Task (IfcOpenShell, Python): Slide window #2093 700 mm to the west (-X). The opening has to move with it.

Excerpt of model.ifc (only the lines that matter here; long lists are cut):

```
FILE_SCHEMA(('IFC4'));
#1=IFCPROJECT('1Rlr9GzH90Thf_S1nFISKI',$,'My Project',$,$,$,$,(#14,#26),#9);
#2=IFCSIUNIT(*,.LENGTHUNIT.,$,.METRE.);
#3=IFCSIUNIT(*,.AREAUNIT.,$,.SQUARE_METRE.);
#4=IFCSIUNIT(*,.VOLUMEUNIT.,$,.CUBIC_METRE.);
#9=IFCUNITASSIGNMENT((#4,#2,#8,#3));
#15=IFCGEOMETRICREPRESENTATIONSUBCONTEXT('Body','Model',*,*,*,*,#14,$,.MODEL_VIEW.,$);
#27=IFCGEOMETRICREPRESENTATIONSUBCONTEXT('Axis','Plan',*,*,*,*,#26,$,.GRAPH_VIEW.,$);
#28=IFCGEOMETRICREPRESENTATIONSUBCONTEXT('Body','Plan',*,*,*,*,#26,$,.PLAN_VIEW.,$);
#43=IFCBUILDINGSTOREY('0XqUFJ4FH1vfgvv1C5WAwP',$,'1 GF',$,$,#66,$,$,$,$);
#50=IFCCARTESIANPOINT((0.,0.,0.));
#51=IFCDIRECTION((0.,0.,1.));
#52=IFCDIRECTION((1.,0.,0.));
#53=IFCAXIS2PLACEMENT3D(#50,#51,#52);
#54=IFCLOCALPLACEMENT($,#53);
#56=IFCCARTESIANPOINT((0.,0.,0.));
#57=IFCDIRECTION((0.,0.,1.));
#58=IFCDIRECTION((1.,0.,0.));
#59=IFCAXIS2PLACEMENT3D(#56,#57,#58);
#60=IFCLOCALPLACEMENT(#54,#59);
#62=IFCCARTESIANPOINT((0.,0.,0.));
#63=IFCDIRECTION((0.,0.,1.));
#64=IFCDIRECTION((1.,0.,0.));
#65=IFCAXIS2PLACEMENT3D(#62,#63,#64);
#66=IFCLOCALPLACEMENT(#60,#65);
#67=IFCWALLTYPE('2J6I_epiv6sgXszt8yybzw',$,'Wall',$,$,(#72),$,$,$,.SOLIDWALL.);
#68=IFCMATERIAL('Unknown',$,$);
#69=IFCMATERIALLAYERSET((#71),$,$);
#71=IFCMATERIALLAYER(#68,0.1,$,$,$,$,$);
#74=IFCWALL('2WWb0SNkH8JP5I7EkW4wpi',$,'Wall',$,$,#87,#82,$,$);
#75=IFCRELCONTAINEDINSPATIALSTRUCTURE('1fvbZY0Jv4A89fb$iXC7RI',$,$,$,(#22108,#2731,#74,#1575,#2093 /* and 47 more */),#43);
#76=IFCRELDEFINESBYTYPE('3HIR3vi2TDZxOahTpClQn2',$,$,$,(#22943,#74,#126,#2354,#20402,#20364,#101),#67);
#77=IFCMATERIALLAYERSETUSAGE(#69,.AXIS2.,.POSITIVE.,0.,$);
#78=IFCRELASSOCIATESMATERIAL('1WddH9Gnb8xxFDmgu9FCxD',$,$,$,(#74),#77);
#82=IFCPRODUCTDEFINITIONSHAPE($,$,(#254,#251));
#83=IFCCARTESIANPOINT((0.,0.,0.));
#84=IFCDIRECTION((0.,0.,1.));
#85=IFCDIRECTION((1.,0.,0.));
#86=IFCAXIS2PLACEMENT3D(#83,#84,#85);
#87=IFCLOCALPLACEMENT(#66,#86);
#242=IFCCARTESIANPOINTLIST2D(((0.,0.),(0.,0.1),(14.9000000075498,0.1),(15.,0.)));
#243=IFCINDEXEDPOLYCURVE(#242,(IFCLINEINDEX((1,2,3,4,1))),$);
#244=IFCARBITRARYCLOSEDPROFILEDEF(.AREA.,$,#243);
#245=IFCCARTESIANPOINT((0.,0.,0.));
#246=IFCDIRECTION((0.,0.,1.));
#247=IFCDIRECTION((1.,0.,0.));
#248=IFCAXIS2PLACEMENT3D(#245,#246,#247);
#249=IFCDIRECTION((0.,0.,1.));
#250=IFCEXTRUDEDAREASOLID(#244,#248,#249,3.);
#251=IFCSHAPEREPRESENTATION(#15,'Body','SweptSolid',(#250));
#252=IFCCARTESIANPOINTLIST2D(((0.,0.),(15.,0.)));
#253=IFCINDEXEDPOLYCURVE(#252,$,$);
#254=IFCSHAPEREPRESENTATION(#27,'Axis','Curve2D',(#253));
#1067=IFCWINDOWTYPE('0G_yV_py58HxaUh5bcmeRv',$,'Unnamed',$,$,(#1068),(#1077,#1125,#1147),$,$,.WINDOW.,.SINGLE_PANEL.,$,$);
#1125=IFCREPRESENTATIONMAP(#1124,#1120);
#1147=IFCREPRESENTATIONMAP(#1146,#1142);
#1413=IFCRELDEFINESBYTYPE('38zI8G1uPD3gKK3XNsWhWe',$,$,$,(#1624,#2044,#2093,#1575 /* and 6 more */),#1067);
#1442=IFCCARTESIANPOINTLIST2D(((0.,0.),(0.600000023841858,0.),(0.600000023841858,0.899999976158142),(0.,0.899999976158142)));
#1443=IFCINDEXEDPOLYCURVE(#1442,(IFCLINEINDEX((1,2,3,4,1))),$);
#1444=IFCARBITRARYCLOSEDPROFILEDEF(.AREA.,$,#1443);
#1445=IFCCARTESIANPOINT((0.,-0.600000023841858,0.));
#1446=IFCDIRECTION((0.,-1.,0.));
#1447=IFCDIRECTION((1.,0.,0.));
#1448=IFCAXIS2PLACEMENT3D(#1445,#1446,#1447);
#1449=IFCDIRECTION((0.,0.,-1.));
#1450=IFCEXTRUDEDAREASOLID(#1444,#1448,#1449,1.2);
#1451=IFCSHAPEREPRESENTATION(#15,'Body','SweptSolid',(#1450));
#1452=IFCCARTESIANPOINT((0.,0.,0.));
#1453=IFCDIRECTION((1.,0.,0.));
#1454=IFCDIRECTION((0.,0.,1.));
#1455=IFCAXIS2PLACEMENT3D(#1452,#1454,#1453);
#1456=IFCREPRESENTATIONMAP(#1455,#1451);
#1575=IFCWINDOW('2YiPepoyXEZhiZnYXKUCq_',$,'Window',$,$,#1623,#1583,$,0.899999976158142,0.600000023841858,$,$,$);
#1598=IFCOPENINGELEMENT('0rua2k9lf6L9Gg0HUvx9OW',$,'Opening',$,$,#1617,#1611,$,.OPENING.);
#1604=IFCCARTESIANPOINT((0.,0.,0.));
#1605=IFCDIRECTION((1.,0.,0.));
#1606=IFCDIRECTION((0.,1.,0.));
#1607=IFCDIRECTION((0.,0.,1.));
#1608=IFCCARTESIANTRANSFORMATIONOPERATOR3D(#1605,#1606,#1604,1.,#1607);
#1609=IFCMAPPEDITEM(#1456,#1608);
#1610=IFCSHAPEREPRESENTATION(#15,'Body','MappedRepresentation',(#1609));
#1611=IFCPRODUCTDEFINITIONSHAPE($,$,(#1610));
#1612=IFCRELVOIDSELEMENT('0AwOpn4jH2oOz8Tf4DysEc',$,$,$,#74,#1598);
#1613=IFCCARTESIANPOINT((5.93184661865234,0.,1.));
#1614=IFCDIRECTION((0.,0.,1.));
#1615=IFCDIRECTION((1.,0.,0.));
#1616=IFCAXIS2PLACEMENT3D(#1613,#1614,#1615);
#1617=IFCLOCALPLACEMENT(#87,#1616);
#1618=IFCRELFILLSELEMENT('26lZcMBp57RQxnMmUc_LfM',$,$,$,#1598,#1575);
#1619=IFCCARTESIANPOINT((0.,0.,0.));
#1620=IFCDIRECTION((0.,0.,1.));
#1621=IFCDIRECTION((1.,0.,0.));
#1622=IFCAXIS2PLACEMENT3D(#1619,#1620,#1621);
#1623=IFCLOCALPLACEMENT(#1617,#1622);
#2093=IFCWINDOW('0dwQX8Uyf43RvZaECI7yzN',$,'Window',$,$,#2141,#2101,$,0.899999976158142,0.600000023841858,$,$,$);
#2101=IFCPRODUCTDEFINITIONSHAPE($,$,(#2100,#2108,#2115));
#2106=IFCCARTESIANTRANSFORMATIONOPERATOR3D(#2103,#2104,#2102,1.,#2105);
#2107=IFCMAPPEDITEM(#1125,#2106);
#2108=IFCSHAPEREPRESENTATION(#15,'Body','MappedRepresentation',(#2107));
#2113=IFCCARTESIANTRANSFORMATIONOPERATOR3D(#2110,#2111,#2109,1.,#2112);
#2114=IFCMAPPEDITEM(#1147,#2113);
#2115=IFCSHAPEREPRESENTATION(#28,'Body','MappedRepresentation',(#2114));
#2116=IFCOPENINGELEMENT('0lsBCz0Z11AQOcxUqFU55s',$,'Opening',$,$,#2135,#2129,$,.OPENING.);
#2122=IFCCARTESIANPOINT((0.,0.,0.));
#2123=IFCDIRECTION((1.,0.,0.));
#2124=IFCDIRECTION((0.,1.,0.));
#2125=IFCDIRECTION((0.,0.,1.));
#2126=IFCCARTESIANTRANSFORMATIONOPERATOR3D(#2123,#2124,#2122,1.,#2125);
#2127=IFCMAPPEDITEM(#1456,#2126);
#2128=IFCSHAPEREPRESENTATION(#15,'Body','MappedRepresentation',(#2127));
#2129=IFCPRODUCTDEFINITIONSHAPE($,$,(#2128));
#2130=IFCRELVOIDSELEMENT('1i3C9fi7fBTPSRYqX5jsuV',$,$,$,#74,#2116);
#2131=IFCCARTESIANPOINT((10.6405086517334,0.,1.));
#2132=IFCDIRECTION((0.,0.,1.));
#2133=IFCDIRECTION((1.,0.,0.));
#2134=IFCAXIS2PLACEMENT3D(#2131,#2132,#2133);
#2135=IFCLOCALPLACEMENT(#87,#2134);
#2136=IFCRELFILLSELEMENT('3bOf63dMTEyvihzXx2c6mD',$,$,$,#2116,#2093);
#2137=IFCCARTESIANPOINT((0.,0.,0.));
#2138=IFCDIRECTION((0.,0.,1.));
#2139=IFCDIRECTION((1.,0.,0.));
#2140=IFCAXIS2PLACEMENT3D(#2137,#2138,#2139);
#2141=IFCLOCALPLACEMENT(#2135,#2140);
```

```python
import ifcopenshell
import ifcopenshell.api.geometry
import ifcopenshell.util.placement
import ifcopenshell.util.unit

model = ifcopenshell.open("model.ifc")
unit_scale = ifcopenshell.util.unit.calculate_unit_scale(model)

window = model.by_id(2093)
opening = window.FillsVoids[0].RelatingOpeningElement
wall = opening.VoidsElements[0].RelatingBuildingElement

wall_matrix = ifcopenshell.util.placement.get_local_placement(wall.ObjectPlacement)
shift = wall_matrix[:3, 0] * -0.7 / unit_scale
before = ifcopenshell.util.placement.get_local_placement(window.ObjectPlacement)[:3, 3].copy()

# The window is placed relative to its opening, so it follows when the opening moves.
matrix = ifcopenshell.util.placement.get_local_placement(opening.ObjectPlacement)
matrix[:3, 3] += shift
ifcopenshell.api.geometry.edit_object_placement(
    model, product=opening, matrix=matrix, is_si=False, should_transform_children=True
)

after = ifcopenshell.util.placement.get_local_placement(window.ObjectPlacement)[:3, 3]
print("window moved by", (after - before).round(3) + 0.0)

model.write("model_updated.ifc")
```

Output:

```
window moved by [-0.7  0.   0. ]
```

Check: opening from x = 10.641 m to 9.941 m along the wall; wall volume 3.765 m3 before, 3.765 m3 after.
